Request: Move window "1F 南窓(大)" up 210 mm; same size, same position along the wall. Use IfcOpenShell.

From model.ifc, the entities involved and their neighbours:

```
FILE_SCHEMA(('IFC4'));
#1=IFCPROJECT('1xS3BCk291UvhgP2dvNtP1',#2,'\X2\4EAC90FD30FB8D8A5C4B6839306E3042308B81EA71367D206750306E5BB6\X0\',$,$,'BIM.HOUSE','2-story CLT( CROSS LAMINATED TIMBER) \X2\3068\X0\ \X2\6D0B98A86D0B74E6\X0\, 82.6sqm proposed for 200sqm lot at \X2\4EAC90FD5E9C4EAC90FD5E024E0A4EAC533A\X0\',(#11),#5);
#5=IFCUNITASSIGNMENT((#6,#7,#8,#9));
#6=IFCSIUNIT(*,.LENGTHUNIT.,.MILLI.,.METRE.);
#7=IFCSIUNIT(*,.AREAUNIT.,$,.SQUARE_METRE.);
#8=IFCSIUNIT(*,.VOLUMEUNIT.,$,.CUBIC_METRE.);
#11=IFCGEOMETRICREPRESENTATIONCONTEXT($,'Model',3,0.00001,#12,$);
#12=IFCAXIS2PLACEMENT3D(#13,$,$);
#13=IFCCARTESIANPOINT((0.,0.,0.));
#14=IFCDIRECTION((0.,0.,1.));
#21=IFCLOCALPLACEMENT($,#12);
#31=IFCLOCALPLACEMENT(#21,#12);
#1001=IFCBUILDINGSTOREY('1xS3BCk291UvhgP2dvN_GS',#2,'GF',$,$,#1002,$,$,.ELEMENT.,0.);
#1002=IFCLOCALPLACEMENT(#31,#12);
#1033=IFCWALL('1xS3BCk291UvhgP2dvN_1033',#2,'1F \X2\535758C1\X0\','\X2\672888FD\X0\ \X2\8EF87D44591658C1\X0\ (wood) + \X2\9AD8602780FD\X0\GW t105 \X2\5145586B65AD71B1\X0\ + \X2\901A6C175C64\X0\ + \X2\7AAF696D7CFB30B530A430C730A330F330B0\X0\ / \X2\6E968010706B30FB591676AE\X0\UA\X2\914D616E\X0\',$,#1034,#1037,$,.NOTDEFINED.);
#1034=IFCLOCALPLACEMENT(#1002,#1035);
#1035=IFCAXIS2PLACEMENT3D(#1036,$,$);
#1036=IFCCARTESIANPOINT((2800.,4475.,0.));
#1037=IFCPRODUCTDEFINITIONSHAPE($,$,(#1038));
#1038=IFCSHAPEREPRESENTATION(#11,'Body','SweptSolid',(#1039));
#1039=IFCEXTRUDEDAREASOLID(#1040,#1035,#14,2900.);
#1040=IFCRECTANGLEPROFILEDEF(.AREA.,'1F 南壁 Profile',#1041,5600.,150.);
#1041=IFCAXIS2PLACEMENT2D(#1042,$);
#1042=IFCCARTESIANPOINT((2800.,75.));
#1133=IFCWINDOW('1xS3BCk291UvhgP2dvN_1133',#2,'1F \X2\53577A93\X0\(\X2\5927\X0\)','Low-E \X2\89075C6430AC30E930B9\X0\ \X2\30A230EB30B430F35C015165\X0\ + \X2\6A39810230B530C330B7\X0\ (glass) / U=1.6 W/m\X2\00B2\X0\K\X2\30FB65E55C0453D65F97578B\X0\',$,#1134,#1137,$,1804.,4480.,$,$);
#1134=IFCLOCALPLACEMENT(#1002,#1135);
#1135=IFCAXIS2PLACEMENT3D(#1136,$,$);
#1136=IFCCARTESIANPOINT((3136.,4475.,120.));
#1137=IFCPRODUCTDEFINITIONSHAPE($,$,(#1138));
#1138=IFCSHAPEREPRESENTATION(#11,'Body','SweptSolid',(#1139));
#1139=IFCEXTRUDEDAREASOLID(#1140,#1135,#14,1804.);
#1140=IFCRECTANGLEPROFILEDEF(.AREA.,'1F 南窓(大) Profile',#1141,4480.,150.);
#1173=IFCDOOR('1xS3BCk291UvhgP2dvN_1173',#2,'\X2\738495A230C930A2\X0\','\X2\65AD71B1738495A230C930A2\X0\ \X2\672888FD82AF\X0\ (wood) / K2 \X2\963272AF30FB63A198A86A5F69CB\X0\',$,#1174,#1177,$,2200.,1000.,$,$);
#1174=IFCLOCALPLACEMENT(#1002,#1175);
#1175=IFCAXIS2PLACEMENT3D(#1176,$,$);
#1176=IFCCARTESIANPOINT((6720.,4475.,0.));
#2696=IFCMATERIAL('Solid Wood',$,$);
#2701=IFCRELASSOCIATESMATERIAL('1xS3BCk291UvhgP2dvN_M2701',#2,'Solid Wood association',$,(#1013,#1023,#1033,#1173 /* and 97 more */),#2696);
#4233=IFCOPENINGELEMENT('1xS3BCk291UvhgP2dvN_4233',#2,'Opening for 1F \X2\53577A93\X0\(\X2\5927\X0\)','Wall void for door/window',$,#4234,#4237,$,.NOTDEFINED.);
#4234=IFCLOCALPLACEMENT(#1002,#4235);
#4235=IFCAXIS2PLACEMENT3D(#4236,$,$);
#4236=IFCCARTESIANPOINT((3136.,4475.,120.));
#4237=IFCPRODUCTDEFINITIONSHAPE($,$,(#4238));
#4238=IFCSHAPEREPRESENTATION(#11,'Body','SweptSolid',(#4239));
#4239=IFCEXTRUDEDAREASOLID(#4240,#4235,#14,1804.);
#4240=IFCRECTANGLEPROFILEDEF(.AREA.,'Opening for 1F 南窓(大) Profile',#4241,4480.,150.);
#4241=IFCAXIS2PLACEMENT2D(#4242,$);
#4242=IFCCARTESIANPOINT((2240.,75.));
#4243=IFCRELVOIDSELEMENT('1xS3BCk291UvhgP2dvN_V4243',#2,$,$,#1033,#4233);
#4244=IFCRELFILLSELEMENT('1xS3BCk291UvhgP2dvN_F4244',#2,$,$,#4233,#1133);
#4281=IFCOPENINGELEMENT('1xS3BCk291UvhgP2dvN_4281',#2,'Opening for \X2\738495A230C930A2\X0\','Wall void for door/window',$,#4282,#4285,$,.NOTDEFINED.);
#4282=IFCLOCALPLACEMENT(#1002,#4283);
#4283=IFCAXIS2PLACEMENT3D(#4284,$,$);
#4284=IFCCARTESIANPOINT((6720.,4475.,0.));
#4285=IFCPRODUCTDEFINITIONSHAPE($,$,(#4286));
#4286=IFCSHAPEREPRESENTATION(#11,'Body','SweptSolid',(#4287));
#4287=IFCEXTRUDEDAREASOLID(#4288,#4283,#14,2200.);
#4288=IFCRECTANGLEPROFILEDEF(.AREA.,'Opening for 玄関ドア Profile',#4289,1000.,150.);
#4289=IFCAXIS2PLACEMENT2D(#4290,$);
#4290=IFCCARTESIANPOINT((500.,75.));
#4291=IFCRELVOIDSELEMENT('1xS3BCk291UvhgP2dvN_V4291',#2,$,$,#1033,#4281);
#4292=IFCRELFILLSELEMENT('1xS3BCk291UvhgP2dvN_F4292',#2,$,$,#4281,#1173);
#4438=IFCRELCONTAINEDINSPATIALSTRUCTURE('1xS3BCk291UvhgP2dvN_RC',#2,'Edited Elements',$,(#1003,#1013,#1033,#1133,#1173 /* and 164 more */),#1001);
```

```python
import numpy as np
import ifcopenshell
import ifcopenshell.api.geometry
import ifcopenshell.util.placement
import ifcopenshell.util.unit

model = ifcopenshell.open("model.ifc")
unit_scale = ifcopenshell.util.unit.calculate_unit_scale(model)

window = model.by_guid("1xS3BCk291UvhgP2dvN_1133")
opening = window.FillsVoids[0].RelatingOpeningElement
dz = 210.0

shift = np.array([0.0, 0.0, dz])
# The window is not placed relative to its opening, so move both.
for product in (opening, window):
    matrix = ifcopenshell.util.placement.get_local_placement(product.ObjectPlacement)
    matrix[:3, 3] += shift
    ifcopenshell.api.geometry.edit_object_placement(model, product=product, matrix=matrix, is_si=False)

print(f"moved by {dz * unit_scale:+.3f} m")

model.write("model-out.ifc")
```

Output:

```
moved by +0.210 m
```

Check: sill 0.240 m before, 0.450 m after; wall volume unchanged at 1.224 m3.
